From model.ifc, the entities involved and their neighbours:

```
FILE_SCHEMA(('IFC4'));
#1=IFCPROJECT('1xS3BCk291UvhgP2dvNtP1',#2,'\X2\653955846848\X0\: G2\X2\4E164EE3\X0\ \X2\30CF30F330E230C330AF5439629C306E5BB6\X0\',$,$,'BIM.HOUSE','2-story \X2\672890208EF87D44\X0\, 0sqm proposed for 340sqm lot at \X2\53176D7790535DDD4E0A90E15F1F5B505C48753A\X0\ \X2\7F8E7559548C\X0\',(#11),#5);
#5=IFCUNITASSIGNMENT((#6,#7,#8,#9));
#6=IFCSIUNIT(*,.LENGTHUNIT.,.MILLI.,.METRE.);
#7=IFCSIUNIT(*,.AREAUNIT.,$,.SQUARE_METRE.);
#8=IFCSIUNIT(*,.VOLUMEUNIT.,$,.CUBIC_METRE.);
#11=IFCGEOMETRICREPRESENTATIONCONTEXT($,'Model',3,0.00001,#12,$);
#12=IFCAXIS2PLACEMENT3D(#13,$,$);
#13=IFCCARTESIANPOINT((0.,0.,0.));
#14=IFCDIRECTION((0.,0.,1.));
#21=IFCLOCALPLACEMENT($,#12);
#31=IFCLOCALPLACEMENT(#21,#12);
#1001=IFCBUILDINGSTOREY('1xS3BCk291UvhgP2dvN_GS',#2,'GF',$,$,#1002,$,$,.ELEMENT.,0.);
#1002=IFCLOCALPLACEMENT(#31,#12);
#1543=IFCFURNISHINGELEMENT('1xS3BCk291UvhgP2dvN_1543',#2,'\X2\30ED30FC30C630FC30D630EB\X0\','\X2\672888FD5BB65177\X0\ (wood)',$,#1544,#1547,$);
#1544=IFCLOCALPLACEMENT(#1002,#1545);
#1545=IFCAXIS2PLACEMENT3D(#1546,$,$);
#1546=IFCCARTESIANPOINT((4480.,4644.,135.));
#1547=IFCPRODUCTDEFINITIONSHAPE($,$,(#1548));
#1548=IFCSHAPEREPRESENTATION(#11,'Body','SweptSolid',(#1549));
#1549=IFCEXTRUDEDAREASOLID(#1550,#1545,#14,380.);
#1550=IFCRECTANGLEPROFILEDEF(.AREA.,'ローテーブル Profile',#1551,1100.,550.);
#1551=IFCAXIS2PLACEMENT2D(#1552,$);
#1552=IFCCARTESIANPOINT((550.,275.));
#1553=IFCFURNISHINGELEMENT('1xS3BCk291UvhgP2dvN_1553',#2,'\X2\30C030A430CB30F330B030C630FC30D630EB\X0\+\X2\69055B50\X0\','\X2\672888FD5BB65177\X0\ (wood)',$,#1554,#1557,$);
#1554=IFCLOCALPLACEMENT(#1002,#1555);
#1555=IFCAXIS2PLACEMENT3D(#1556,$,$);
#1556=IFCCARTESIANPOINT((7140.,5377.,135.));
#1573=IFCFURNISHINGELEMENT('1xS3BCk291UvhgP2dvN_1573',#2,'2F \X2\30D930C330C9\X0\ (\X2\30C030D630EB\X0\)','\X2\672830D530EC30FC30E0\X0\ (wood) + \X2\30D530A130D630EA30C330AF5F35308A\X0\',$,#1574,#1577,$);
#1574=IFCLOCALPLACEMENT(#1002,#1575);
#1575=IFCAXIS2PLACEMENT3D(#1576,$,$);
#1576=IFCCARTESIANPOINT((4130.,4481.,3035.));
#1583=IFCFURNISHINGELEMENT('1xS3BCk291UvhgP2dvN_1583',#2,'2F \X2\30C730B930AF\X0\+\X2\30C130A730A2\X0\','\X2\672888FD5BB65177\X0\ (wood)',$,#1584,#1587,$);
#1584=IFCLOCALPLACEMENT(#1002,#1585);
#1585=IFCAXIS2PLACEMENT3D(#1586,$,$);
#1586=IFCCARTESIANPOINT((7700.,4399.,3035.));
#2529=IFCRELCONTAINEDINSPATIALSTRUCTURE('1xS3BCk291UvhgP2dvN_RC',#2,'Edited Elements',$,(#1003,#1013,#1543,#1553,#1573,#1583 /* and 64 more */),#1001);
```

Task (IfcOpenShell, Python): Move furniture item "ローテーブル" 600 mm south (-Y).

```python
import ifcopenshell
import ifcopenshell.api.geometry
import ifcopenshell.util.placement
import ifcopenshell.util.unit

model = ifcopenshell.open("model.ifc")
unit_scale = ifcopenshell.util.unit.calculate_unit_scale(model)

item = model.by_guid("1xS3BCk291UvhgP2dvN_1543")
matrix = ifcopenshell.util.placement.get_local_placement(item.ObjectPlacement)
matrix[1, 3] -= 0.6 / unit_scale
ifcopenshell.api.geometry.edit_object_placement(model, product=item, matrix=matrix, is_si=False)

print(ifcopenshell.util.placement.get_local_placement(item.ObjectPlacement).round(3) + 0.0)

model.write("model_updated.ifc")
```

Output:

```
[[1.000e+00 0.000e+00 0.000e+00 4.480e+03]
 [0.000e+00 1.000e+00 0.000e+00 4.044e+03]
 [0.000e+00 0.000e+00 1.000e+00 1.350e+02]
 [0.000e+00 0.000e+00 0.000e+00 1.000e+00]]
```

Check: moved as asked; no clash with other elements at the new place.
